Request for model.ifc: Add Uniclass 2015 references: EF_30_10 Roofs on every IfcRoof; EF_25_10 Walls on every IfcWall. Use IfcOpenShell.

First a look at what the model holds.

```python
import ifcopenshell

model = ifcopenshell.open("model.ifc")
print(model.schema)
print("classifications:", [c.Name for c in model.by_type("IfcClassification")])
for ifc_class in ("IfcDoor", "IfcRoof", "IfcStair", "IfcWall", "IfcWindow"):
    print(ifc_class, len(model.by_type(ifc_class)))
```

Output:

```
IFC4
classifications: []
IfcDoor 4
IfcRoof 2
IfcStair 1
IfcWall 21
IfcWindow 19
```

```python
import ifcopenshell
import ifcopenshell.api.classification

model = ifcopenshell.open("model.ifc")

system = ifcopenshell.api.classification.add_classification(model, classification="Uniclass 2015")

codes = {
    "IfcRoof": ("EF_30_10", "Roofs"),
    "IfcWall": ("EF_25_10", "Walls"),
}
for ifc_class, (code, name) in codes.items():
    products = model.by_type(ifc_class)
    ifcopenshell.api.classification.add_reference(
        model, products=products, classification=system, identification=code, name=name
    )
    print(code, len(products))

model.write("model_updated.ifc")
```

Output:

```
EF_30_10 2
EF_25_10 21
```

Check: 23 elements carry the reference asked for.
